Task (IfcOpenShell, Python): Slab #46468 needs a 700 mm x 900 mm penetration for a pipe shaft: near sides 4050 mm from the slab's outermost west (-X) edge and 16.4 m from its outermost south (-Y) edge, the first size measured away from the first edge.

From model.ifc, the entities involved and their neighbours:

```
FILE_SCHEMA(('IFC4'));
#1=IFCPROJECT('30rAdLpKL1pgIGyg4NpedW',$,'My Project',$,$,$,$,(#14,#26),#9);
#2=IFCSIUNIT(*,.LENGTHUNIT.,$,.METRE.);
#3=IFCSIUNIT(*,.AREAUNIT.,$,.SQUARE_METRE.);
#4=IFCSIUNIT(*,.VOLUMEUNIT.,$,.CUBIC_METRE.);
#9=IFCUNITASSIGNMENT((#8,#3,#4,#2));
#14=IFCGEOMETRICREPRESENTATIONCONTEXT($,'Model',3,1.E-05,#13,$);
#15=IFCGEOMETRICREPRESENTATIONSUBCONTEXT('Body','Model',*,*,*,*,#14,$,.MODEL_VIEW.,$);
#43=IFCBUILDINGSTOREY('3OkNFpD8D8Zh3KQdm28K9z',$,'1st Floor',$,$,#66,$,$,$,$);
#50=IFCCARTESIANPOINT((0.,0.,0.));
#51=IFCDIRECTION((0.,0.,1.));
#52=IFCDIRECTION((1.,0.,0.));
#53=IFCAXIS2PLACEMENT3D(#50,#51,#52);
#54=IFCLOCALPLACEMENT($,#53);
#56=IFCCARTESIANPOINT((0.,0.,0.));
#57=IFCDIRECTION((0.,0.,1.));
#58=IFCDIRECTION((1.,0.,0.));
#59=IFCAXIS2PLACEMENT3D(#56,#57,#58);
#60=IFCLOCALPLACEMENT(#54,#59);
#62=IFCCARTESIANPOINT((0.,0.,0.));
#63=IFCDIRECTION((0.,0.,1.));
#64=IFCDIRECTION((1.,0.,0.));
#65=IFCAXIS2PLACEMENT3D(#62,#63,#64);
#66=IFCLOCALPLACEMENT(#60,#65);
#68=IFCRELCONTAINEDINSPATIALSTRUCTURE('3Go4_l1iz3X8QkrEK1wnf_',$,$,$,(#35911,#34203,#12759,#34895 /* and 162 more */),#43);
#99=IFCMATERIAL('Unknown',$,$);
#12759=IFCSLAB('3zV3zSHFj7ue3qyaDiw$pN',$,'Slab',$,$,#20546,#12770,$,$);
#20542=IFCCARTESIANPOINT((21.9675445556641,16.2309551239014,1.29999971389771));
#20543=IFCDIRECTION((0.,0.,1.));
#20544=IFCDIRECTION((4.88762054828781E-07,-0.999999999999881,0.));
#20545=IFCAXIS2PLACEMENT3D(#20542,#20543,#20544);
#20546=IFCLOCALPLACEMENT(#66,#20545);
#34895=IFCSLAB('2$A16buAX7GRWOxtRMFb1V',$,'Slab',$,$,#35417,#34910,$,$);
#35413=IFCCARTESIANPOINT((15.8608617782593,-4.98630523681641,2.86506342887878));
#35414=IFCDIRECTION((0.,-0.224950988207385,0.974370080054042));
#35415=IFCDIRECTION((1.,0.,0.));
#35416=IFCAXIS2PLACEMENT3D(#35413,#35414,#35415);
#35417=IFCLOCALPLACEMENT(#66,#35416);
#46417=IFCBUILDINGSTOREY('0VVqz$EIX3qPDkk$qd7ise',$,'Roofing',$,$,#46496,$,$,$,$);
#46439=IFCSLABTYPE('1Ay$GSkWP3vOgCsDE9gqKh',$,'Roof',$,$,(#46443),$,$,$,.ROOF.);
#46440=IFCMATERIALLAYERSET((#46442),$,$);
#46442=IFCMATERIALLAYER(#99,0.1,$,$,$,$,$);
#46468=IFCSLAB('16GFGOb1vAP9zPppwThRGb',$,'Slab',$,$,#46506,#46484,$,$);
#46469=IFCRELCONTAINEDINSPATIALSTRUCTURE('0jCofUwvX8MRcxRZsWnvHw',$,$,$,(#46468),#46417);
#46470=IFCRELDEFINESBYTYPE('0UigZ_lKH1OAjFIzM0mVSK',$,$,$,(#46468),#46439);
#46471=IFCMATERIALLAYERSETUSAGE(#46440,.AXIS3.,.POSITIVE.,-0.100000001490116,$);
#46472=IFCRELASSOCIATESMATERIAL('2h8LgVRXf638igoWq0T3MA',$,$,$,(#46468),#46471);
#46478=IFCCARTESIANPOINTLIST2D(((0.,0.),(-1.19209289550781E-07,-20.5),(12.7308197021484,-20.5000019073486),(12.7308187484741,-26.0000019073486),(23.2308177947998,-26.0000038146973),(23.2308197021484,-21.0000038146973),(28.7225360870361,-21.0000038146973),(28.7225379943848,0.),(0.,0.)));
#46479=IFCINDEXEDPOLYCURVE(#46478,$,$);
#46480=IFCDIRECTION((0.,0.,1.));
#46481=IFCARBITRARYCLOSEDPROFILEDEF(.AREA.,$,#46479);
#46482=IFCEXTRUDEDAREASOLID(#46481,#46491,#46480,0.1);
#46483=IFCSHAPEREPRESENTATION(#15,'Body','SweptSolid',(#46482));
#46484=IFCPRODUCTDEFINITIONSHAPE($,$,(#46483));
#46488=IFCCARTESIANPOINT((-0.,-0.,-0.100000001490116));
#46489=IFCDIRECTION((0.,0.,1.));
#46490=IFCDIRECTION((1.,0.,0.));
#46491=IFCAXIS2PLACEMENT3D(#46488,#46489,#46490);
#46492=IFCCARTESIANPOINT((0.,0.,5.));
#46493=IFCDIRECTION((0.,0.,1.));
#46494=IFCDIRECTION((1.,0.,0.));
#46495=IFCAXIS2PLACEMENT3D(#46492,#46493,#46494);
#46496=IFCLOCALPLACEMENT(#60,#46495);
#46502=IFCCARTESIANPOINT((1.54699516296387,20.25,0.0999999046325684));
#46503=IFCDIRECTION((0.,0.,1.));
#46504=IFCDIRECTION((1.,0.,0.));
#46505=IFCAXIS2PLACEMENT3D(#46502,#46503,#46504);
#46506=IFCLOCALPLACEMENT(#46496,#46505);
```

```python
import numpy as np
import ifcopenshell
import ifcopenshell.api.feature
import ifcopenshell.api.geometry
import ifcopenshell.api.root
import ifcopenshell.geom
import ifcopenshell.util.placement
import ifcopenshell.util.representation
import ifcopenshell.util.shape
import ifcopenshell.util.unit

model = ifcopenshell.open("model.ifc")
unit_scale = ifcopenshell.util.unit.calculate_unit_scale(model)
settings = ifcopenshell.geom.settings()


def volume(element):
    """Net volume in cubic metres, openings subtracted."""
    shape = ifcopenshell.geom.create_shape(settings, element)
    return ifcopenshell.util.shape.get_volume(shape.geometry)


slab = model.by_guid("16GFGOb1vAP9zPppwThRGb")
before = volume(slab)

# Extent in the slab's own axes, in metres. The edges named are its -X and -Y sides.
slab_shape = ifcopenshell.geom.create_shape(settings, slab)
vertices = ifcopenshell.util.shape.get_vertices(slab_shape.geometry)
x_min, y_min, bottom = vertices.min(axis=0)
top = vertices[:, 2].max()

opening = ifcopenshell.api.root.create_entity(model, ifc_class="IfcOpeningElement", name="Pipe shaft opening", predefined_type="OPENING")
context = ifcopenshell.util.representation.get_context(model, "Model", "Body", "MODEL_VIEW")
width, depth = 0.7, 0.9
outline = [(0.0, 0.0), (width, 0.0), (width, depth), (0.0, depth), (0.0, 0.0)]
# Overshoot both faces by 50 mm so the cut is clean.
shape = ifcopenshell.api.geometry.add_slab_representation(
    model, context=context, depth=top - bottom + 0.1, polyline=outline
)
ifcopenshell.api.geometry.assign_representation(model, product=opening, representation=shape)

matrix = ifcopenshell.util.placement.get_local_placement(slab.ObjectPlacement)
matrix[:, 3] = matrix @ np.append(np.array([x_min + 4.05, y_min + 16.4, bottom - 0.05]) / unit_scale, 1.0)
ifcopenshell.api.geometry.edit_object_placement(model, product=opening, matrix=matrix, is_si=False)
ifcopenshell.api.feature.add_feature(model, feature=opening, element=slab)

after = volume(slab)

print(f"slab volume {before:.3f} -> {after:.3f} m3")

model.write("model_edited.ifc")
```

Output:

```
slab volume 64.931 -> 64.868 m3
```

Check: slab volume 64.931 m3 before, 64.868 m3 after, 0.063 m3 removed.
